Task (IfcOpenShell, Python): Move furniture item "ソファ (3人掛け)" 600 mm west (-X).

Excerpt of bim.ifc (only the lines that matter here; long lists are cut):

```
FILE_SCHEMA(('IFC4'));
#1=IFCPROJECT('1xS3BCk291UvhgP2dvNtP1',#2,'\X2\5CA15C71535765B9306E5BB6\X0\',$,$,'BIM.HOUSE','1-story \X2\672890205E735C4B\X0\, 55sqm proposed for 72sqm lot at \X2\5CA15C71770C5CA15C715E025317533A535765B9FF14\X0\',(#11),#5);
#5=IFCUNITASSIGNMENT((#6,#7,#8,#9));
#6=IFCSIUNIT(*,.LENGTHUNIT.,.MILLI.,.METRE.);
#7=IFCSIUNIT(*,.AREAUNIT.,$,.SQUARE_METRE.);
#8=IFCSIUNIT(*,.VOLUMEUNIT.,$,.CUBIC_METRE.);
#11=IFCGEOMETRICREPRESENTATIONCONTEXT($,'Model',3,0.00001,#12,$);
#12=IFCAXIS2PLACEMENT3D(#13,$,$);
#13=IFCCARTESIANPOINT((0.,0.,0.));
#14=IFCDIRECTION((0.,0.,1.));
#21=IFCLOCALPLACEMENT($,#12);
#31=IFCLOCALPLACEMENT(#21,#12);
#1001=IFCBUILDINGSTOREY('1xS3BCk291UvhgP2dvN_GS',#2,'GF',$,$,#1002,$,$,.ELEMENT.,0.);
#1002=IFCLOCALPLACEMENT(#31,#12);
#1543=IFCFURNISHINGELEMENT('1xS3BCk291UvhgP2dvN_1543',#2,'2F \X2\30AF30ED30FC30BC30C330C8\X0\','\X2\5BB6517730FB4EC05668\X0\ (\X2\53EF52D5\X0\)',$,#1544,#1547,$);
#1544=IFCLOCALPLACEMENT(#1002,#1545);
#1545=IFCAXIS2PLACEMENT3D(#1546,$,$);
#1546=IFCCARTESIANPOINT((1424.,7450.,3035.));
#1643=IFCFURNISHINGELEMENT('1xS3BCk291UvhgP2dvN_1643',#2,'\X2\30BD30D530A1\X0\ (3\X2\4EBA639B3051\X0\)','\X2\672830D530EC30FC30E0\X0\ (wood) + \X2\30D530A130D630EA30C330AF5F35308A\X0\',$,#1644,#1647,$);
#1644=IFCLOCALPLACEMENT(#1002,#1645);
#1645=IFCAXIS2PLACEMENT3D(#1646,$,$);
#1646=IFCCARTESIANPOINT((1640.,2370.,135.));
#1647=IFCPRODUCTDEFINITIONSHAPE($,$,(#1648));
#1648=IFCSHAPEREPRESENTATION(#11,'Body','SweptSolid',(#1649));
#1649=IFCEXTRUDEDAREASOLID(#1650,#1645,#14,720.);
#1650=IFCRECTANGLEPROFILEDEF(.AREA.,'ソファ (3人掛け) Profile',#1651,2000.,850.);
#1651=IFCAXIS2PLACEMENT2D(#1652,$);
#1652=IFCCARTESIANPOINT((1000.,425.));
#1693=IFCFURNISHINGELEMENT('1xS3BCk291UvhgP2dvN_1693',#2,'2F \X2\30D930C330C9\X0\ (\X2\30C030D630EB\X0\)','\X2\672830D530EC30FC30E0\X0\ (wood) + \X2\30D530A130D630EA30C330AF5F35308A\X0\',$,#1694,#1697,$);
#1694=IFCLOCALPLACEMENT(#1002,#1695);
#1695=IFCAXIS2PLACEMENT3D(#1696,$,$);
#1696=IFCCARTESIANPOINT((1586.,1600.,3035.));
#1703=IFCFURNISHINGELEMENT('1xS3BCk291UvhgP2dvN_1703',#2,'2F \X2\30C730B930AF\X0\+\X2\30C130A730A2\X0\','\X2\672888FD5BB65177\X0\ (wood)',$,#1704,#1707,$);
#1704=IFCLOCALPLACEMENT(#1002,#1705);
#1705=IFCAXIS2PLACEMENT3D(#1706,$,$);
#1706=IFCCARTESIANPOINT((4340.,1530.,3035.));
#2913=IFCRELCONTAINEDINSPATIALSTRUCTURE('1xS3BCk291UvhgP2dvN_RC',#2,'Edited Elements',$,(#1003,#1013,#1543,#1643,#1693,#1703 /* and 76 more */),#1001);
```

```python
import ifcopenshell
import ifcopenshell.api.geometry
import ifcopenshell.util.placement
import ifcopenshell.util.unit

model = ifcopenshell.open("bim.ifc")
unit_scale = ifcopenshell.util.unit.calculate_unit_scale(model)

item = model.by_id(1643)
matrix = ifcopenshell.util.placement.get_local_placement(item.ObjectPlacement)
matrix[0, 3] -= 0.6 / unit_scale
ifcopenshell.api.geometry.edit_object_placement(model, product=item, matrix=matrix, is_si=False)

print(ifcopenshell.util.placement.get_local_placement(item.ObjectPlacement).round(3) + 0.0)

model.write("bim_updated.ifc")
```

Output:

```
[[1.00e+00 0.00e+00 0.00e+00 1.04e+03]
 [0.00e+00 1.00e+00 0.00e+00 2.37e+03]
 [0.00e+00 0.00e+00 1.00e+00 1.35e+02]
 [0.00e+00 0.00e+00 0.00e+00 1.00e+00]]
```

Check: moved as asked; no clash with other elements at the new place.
